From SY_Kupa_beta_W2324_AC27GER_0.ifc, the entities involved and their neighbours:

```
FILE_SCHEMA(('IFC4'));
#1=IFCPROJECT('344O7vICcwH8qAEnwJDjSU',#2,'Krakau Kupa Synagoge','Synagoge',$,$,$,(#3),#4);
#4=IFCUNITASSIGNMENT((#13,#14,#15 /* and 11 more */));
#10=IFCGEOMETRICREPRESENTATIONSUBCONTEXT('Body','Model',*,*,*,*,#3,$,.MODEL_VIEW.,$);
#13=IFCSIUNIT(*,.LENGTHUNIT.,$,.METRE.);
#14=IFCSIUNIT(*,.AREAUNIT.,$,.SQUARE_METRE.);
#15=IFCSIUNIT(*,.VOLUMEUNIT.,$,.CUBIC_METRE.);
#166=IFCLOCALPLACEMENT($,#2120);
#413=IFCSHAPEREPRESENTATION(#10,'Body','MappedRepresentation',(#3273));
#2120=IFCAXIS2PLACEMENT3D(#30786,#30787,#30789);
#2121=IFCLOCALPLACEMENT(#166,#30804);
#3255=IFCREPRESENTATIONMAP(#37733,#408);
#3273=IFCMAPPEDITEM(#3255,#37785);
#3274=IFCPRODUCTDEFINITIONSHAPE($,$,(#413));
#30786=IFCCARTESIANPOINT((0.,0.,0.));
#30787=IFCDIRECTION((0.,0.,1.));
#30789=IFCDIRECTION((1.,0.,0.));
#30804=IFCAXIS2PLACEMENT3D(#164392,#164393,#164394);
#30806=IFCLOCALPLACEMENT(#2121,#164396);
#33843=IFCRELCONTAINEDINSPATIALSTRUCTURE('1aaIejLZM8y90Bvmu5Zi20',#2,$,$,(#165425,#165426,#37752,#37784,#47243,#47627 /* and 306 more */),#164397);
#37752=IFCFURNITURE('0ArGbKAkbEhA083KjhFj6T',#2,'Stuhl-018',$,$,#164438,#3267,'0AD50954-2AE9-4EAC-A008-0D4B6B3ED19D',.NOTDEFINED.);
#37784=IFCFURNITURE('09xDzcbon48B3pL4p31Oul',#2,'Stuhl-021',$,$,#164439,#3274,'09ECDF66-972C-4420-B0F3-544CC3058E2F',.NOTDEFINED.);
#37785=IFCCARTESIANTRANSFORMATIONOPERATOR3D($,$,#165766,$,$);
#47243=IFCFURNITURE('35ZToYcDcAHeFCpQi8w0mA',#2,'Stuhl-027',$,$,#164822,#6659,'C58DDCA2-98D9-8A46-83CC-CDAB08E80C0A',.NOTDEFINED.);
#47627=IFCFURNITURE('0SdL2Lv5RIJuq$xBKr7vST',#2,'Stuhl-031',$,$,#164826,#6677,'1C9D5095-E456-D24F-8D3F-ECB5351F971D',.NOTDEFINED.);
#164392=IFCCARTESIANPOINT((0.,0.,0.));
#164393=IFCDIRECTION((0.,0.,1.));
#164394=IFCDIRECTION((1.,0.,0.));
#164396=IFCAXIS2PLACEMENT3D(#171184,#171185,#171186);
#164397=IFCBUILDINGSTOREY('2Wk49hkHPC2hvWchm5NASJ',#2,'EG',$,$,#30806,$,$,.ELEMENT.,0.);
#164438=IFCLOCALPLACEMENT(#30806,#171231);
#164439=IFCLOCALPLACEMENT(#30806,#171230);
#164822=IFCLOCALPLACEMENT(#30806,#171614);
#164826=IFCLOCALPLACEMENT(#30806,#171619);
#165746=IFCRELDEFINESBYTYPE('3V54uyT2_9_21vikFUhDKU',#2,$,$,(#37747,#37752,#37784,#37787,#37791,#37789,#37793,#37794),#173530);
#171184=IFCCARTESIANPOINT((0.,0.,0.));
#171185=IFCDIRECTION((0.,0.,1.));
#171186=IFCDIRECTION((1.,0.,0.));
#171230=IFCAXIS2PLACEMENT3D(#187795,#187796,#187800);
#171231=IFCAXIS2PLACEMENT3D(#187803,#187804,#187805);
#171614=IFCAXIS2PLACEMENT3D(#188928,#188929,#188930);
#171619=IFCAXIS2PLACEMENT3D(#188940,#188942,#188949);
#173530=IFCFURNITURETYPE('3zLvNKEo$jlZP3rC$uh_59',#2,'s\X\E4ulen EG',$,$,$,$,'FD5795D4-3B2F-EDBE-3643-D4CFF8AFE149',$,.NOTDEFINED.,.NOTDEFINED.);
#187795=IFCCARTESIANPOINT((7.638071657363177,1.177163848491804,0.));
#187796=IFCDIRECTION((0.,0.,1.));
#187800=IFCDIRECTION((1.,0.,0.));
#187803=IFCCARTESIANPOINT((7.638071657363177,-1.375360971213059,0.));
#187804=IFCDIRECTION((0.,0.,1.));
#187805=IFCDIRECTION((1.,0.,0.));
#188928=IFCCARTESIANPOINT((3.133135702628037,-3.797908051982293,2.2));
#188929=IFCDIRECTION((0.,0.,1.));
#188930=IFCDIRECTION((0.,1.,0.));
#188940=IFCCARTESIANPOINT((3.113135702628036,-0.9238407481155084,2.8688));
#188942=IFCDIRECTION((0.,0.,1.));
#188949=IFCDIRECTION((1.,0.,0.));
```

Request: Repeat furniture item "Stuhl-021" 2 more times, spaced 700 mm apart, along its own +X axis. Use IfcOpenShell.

```python
import ifcopenshell
import ifcopenshell.api.geometry
import ifcopenshell.api.root
import ifcopenshell.util.element
import ifcopenshell.util.placement
import ifcopenshell.util.unit

model = ifcopenshell.open("SY_Kupa_beta_W2324_AC27GER_0.ifc")
unit_scale = ifcopenshell.util.unit.calculate_unit_scale(model)


def reuse_history(source, copy):
    """copy_class also copies each property set's owner history, people and application; keep the originals."""
    for rel in copy.IsDefinedBy:
        if rel.is_a("IfcRelDefinesByProperties") and (history := rel.RelatingPropertyDefinition.OwnerHistory):
            rel.RelatingPropertyDefinition.OwnerHistory = source.OwnerHistory
            ifcopenshell.util.element.remove_deep2(model, history)


source = model.by_guid("09xDzcbon48B3pL4p31Oul")
base = ifcopenshell.util.placement.get_local_placement(source.ObjectPlacement)
step = base[:3, 0] * 0.7 / unit_scale

for i in range(1, 3):
    copy = ifcopenshell.api.root.copy_class(model, product=source)
    copy.Representation = ifcopenshell.util.element.copy_deep(
        model, source.Representation, exclude=["IfcGeometricRepresentationContext", "IfcRepresentationMap"]
    )
    copy.Tag = None
    reuse_history(source, copy)
    matrix = base.copy()
    matrix[:3, 3] += i * step
    print("added at", matrix[:3, 3].round(3) + 0.0)
    ifcopenshell.api.geometry.edit_object_placement(model, product=copy, matrix=matrix, is_si=False)

model.write("SY_Kupa_beta_W2324_AC27GER_0_updated.ifc")
```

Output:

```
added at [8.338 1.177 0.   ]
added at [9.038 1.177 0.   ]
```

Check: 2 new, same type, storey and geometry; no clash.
